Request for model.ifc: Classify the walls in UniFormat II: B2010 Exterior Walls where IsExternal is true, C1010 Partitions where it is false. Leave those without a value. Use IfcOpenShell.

First a look at what the model holds.

```python
import ifcopenshell
import ifcopenshell.util.element

model = ifcopenshell.open("model.ifc")
print(model.schema)
print("classifications:", [c.Name for c in model.by_type("IfcClassification")])
values = [ifcopenshell.util.element.get_pset(e, "Pset_WallCommon", "IsExternal") for e in model.by_type("IfcWall")]
for value in (True, False, None):
    print("IsExternal", value, values.count(value))
```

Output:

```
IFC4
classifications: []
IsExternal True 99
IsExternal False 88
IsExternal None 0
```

```python
import ifcopenshell
import ifcopenshell.api.classification
import ifcopenshell.util.element

model = ifcopenshell.open("model.ifc")

system = ifcopenshell.api.classification.add_classification(model, classification="UniFormat II")

walls = model.by_type("IfcWall")
external = {e: ifcopenshell.util.element.get_pset(e, "Pset_WallCommon", "IsExternal") for e in walls}
for flag, code, name in ((True, "B2010", "Exterior Walls"), (False, "C1010", "Partitions")):
    products = [e for e in walls if external[e] is flag]
    ifcopenshell.api.classification.add_reference(
        model, products=products, classification=system, identification=code, name=name
    )
    print(code, len(products))

model.write("model_rev.ifc")
```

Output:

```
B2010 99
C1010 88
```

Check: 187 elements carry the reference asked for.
